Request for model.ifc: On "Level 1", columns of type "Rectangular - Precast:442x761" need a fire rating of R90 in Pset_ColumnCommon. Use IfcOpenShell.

First a look at what the model holds.

```python
import ifcopenshell
import ifcopenshell.util.element

model = ifcopenshell.open("model.ifc")
print(model.schema)
storey = next(s for s in model.by_type("IfcBuildingStorey") if s.Name == "Level 1")
columns = [e for e in ifcopenshell.util.element.get_decomposition(storey) if e.is_a("IfcColumn")]
seen = {}
for e in columns:
    element_type = ifcopenshell.util.element.get_type(e)
    key = (element_type.Name if element_type != e and element_type else None, ifcopenshell.util.element.get_pset(e, "Pset_ColumnCommon", "FireRating"))
    seen[key] = seen.get(key, 0) + 1
for (name, value), count in sorted(seen.items(), key=str):
    print(count, "x", name, "|", value)
```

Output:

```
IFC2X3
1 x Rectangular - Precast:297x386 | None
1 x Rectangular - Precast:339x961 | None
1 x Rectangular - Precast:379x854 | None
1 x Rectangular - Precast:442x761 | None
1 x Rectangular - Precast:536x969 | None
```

```python
import ifcopenshell
import ifcopenshell.api.pset
import ifcopenshell.util.element

model = ifcopenshell.open("model.ifc")

storey = next(s for s in model.by_type("IfcBuildingStorey") if s.Name == "Level 1")
columns = [e for e in ifcopenshell.util.element.get_decomposition(storey) if e.is_a("IfcColumn")]

count = 0
for e in columns:
    element_type = ifcopenshell.util.element.get_type(e)
    if element_type in (None, e) or element_type.Name != "Rectangular - Precast:442x761":
        continue
    # add_pset returns the element's existing set when there is one.
    pset = ifcopenshell.api.pset.add_pset(model, product=e, name="Pset_ColumnCommon")
    ifcopenshell.api.pset.edit_pset(model, pset=pset, properties={"FireRating": "R90"})
    count += 1

print(count, "columns updated")

model.write("model_edited.ifc")
```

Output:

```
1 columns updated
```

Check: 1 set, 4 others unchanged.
